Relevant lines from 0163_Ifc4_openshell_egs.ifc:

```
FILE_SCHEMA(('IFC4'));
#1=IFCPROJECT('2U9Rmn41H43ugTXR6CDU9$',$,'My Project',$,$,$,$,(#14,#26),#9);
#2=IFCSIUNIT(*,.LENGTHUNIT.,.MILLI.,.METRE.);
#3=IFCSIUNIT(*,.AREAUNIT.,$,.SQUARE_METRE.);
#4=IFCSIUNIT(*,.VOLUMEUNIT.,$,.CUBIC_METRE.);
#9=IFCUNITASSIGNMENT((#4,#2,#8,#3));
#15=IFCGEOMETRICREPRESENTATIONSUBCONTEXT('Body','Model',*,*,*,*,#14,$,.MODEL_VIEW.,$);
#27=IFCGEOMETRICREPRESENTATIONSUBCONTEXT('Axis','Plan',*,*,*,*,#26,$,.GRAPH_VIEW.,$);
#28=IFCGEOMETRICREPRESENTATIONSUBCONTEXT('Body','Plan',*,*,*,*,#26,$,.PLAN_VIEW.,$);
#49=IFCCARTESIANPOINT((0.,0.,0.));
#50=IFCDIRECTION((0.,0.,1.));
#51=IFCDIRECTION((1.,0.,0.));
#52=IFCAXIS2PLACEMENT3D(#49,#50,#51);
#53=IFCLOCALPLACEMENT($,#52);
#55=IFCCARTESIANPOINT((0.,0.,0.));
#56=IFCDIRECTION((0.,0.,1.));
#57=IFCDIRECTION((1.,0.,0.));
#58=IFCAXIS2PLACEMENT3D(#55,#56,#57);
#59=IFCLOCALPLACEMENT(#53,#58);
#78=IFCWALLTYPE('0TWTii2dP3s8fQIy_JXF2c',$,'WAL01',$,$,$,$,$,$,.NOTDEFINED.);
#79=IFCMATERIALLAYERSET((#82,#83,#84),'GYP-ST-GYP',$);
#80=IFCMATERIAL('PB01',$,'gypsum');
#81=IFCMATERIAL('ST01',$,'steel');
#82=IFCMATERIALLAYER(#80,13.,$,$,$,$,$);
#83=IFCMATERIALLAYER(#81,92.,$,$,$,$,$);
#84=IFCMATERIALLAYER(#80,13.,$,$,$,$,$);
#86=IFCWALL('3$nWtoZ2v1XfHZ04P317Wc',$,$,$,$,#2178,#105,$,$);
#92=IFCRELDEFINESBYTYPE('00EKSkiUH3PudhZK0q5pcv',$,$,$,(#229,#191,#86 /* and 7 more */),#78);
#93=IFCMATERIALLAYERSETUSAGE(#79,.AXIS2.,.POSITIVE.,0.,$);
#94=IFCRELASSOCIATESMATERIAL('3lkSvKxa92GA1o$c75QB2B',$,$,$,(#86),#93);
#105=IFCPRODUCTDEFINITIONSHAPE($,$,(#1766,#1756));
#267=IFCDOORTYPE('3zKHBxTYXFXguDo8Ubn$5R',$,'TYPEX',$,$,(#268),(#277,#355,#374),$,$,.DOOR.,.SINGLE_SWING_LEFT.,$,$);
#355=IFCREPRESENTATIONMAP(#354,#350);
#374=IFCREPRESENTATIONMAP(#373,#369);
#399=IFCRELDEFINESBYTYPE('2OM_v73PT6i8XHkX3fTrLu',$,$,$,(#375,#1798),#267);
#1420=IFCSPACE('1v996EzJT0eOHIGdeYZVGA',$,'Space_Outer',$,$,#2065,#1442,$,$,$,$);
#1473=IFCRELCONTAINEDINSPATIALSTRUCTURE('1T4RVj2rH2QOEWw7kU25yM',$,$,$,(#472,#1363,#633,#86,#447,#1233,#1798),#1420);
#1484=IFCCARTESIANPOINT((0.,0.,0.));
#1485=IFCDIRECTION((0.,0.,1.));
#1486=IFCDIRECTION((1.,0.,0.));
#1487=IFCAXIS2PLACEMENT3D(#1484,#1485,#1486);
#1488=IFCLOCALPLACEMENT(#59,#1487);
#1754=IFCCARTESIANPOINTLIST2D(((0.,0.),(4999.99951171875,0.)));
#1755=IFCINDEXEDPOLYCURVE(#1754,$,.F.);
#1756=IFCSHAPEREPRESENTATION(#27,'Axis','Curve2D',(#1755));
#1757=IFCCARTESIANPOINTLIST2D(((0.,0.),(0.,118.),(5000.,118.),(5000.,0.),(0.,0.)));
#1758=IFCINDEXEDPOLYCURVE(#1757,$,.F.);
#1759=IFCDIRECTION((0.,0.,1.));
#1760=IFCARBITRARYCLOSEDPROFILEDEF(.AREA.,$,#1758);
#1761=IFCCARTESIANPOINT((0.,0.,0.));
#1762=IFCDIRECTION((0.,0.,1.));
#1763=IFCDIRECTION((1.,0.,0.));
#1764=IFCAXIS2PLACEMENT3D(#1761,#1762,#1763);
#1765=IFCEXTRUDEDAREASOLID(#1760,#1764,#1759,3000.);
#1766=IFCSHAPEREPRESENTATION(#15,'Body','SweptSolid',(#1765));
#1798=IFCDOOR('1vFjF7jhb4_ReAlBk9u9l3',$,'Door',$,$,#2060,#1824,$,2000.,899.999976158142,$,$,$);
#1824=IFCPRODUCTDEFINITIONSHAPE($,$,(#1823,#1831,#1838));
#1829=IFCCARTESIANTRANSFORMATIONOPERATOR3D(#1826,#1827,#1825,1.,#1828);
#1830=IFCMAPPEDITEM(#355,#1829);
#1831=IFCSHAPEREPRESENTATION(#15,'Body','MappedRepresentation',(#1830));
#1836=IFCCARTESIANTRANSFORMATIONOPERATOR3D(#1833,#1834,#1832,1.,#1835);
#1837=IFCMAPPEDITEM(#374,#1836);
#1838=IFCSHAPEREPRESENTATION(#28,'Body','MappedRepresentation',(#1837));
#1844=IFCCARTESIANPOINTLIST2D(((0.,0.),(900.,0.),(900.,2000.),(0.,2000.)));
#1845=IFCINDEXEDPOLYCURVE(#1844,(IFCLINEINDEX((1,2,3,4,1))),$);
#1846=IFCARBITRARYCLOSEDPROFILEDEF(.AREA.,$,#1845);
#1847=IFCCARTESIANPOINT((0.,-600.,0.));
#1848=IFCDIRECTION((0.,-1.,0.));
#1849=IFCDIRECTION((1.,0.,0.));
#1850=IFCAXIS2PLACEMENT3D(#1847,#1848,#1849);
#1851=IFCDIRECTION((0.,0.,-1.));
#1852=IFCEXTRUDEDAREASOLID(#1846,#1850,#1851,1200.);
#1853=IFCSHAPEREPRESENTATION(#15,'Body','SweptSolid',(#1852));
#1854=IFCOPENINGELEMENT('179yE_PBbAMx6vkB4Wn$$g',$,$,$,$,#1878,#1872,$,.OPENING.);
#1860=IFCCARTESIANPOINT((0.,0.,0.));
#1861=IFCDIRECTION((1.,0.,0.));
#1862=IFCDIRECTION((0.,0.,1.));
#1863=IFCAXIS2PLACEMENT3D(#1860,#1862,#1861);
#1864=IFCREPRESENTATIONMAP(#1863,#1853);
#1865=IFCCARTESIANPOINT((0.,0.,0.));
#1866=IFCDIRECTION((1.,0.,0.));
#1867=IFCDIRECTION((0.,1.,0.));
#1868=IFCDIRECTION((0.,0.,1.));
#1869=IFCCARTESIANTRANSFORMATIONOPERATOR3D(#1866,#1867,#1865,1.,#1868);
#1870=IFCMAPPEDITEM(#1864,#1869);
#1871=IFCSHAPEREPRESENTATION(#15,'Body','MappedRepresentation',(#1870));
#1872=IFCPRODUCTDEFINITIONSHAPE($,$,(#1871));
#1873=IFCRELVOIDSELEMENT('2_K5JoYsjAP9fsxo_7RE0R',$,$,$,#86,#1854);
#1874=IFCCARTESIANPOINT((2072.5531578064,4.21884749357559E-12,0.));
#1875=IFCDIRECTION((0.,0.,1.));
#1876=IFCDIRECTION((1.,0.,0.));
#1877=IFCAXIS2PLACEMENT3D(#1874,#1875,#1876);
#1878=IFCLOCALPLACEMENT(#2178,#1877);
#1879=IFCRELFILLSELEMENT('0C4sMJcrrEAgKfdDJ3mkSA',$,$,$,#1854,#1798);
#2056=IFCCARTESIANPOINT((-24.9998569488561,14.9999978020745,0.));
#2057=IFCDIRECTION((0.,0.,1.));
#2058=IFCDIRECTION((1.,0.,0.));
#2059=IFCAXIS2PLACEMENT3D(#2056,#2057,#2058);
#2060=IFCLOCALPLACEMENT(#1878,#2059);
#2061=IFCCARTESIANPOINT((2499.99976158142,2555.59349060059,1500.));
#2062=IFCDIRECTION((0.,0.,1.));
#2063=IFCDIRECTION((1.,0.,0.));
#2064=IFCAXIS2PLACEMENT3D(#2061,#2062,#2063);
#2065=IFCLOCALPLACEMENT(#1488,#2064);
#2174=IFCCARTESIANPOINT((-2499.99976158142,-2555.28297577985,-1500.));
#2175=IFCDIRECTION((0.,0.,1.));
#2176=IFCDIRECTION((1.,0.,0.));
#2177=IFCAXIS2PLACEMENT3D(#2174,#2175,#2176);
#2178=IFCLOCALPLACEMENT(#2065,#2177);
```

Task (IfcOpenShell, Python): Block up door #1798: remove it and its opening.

```python
import ifcopenshell
import ifcopenshell.api.feature
import ifcopenshell.api.root
import ifcopenshell.geom
import ifcopenshell.util.shape

model = ifcopenshell.open("0163_Ifc4_openshell_egs.ifc")
settings = ifcopenshell.geom.settings()


def volume(element):
    """Net volume in cubic metres, openings subtracted."""
    shape = ifcopenshell.geom.create_shape(settings, element)
    return ifcopenshell.util.shape.get_volume(shape.geometry)


door = model.by_guid("1vFjF7jhb4_ReAlBk9u9l3")
opening = door.FillsVoids[0].RelatingOpeningElement
wall = opening.VoidsElements[0].RelatingBuildingElement
before = volume(wall)

ifcopenshell.api.root.remove_product(model, product=door)
ifcopenshell.api.feature.remove_feature(model, feature=opening)

after = volume(wall)

print(f"wall volume {before:.3f} -> {after:.3f} m3")

model.write("0163_Ifc4_openshell_egs_updated.ifc")
```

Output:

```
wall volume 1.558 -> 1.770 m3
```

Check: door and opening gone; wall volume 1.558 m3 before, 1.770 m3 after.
